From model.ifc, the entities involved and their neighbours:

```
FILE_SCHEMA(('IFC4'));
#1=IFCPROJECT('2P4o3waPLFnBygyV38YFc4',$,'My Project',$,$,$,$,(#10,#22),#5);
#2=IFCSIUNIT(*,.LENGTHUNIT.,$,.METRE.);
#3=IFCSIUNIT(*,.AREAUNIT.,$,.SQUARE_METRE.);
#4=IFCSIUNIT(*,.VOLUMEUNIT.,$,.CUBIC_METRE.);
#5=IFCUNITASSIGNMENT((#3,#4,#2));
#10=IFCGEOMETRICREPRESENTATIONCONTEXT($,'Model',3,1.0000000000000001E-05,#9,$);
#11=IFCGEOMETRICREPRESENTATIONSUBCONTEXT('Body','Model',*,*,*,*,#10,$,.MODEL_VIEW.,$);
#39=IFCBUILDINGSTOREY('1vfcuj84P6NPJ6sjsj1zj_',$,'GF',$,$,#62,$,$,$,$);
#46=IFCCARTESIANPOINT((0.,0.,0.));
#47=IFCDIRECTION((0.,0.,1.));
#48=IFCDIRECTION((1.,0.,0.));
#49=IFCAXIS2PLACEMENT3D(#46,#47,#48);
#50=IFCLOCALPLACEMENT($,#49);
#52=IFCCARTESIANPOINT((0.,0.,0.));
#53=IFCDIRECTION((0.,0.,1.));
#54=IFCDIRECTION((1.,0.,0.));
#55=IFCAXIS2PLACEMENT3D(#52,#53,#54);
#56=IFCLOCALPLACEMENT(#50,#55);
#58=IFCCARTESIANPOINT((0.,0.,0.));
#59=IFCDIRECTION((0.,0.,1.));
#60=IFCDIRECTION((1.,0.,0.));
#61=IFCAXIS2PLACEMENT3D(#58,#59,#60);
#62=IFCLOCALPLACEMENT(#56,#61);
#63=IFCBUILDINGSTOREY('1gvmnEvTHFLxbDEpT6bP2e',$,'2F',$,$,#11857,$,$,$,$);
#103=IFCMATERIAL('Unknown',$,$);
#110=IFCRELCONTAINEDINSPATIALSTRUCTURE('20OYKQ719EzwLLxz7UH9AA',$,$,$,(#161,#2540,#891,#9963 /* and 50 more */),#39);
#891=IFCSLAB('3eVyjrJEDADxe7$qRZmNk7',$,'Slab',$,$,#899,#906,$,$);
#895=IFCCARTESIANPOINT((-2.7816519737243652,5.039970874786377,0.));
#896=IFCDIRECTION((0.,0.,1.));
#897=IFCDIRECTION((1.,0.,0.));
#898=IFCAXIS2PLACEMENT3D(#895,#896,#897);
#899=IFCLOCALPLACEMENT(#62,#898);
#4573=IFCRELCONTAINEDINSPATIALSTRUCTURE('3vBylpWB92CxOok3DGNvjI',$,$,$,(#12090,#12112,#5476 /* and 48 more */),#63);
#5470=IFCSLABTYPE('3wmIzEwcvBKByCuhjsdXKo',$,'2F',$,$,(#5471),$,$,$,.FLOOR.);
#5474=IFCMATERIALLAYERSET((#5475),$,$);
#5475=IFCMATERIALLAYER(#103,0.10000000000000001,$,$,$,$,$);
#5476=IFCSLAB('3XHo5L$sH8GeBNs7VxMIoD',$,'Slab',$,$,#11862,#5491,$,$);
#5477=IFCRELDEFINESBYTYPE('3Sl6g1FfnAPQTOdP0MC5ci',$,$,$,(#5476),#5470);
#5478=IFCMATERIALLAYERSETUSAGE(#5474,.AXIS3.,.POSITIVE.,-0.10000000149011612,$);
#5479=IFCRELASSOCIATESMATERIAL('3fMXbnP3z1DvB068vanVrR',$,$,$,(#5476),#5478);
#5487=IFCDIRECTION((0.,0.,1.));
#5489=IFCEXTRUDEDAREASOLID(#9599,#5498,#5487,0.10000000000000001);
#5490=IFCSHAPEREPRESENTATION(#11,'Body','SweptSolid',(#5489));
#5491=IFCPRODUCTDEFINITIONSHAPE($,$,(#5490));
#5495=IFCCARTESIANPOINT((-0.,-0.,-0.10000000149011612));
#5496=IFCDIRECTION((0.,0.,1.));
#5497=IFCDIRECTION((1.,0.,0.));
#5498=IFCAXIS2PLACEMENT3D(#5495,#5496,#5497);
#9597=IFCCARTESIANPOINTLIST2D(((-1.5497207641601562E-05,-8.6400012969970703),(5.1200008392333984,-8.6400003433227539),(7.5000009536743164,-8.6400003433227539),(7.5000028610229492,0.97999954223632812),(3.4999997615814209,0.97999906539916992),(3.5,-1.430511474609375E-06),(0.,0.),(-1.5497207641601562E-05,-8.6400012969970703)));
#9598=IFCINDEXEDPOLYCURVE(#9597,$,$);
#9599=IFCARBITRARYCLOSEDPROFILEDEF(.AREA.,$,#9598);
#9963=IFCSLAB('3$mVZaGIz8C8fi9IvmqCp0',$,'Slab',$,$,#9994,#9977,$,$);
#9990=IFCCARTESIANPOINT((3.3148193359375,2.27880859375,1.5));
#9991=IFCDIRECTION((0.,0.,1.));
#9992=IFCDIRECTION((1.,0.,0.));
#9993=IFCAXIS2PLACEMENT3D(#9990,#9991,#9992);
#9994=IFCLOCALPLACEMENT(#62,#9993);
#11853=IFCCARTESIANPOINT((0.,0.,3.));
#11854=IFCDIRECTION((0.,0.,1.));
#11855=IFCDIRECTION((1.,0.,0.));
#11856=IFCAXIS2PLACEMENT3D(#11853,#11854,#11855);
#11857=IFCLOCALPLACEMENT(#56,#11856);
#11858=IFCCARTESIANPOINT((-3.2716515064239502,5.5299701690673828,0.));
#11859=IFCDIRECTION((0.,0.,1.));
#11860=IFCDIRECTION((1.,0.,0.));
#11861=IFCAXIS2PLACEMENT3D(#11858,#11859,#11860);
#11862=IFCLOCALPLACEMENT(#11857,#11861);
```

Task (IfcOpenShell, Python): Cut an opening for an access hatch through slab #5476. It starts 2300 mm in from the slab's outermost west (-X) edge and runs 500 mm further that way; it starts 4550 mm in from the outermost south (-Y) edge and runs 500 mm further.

```python
import numpy as np
import ifcopenshell
import ifcopenshell.api.feature
import ifcopenshell.api.geometry
import ifcopenshell.api.root
import ifcopenshell.geom
import ifcopenshell.util.placement
import ifcopenshell.util.representation
import ifcopenshell.util.shape
import ifcopenshell.util.unit

model = ifcopenshell.open("model.ifc")
unit_scale = ifcopenshell.util.unit.calculate_unit_scale(model)
settings = ifcopenshell.geom.settings()


def volume(element):
    """Net volume in cubic metres, openings subtracted."""
    shape = ifcopenshell.geom.create_shape(settings, element)
    return ifcopenshell.util.shape.get_volume(shape.geometry)


slab = model.by_guid("3XHo5L$sH8GeBNs7VxMIoD")
before = volume(slab)

# Extent in the slab's own axes, in metres. The edges named are its -X and -Y sides.
slab_shape = ifcopenshell.geom.create_shape(settings, slab)
vertices = ifcopenshell.util.shape.get_vertices(slab_shape.geometry)
x_min, y_min, bottom = vertices.min(axis=0)
top = vertices[:, 2].max()

opening = ifcopenshell.api.root.create_entity(model, ifc_class="IfcOpeningElement", name="Access hatch opening", predefined_type="OPENING")
context = ifcopenshell.util.representation.get_context(model, "Model", "Body", "MODEL_VIEW")
width, depth = 0.5, 0.5
outline = [(0.0, 0.0), (width, 0.0), (width, depth), (0.0, depth), (0.0, 0.0)]
# Overshoot both faces by 50 mm so the cut is clean.
shape = ifcopenshell.api.geometry.add_slab_representation(
    model, context=context, depth=top - bottom + 0.1, polyline=outline
)
ifcopenshell.api.geometry.assign_representation(model, product=opening, representation=shape)

matrix = ifcopenshell.util.placement.get_local_placement(slab.ObjectPlacement)
matrix[:, 3] = matrix @ np.append(np.array([x_min + 2.3, y_min + 4.55, bottom - 0.05]) / unit_scale, 1.0)
ifcopenshell.api.geometry.edit_object_placement(model, product=opening, matrix=matrix, is_si=False)
ifcopenshell.api.feature.add_feature(model, feature=opening, element=slab)

after = volume(slab)

print(f"slab volume {before:.3f} -> {after:.3f} m3")

model.write("model_rev.ifc")
```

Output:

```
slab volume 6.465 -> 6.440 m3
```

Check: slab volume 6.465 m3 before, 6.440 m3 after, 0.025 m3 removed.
